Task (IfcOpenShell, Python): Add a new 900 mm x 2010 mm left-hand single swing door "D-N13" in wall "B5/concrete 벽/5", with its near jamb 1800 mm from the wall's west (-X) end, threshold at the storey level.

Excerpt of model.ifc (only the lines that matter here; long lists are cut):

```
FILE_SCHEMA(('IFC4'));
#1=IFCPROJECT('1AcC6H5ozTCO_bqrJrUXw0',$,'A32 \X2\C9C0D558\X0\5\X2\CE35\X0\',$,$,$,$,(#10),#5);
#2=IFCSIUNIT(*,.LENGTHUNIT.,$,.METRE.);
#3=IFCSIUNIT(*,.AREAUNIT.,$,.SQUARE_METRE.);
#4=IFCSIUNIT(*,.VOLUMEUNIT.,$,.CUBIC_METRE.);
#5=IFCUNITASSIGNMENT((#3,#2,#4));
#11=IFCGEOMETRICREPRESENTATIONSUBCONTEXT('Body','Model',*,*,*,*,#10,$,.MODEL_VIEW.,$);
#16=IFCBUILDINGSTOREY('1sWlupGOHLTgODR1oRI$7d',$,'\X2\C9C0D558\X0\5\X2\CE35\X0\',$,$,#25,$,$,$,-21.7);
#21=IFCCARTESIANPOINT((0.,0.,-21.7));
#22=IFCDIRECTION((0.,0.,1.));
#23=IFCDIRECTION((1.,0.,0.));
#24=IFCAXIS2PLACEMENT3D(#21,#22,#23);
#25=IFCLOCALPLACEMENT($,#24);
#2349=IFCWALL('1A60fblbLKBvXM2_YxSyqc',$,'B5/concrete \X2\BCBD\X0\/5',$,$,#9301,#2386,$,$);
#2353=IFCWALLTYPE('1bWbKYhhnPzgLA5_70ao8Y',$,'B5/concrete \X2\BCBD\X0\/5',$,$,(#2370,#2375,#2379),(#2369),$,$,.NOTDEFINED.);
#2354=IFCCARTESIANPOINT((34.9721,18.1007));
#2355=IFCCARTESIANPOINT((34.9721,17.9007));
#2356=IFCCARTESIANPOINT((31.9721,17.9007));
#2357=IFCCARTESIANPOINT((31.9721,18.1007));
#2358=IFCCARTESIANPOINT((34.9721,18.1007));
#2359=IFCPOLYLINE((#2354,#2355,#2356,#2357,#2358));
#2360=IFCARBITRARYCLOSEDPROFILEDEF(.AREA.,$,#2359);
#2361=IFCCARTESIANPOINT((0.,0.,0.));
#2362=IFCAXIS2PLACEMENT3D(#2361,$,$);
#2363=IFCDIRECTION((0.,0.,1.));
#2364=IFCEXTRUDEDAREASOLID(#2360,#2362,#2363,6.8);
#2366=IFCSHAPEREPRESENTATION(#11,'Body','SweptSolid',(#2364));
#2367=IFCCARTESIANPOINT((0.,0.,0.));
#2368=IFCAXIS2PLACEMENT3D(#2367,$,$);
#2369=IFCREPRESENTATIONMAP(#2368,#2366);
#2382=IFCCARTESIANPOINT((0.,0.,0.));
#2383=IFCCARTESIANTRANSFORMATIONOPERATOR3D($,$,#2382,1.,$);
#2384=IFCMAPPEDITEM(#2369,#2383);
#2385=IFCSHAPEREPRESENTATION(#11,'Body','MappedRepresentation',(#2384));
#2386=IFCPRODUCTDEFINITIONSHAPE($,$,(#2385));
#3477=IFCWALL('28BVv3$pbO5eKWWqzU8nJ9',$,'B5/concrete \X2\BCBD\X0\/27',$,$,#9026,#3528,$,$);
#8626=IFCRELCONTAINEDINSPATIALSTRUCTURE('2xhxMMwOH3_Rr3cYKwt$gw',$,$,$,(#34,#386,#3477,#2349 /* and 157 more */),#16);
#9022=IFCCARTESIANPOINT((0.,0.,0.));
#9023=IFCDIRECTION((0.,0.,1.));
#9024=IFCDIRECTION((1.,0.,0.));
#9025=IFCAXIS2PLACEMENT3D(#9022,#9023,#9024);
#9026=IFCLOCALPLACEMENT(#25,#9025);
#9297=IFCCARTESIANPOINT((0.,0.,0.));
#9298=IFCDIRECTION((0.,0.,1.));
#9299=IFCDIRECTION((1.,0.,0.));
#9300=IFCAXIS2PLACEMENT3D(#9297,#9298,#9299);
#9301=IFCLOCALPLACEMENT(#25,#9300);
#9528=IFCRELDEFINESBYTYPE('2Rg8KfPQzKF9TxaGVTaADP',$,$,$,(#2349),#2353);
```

```python
import numpy as np
import ifcopenshell
import ifcopenshell.api.feature
import ifcopenshell.api.geometry
import ifcopenshell.api.root
import ifcopenshell.api.spatial
import ifcopenshell.geom
import ifcopenshell.util.element
import ifcopenshell.util.placement
import ifcopenshell.util.representation
import ifcopenshell.util.shape
import ifcopenshell.util.unit

model = ifcopenshell.open("model.ifc")
unit_scale = ifcopenshell.util.unit.calculate_unit_scale(model)
settings = ifcopenshell.geom.settings()


def volume(element):
    """Net volume in cubic metres, openings subtracted."""
    shape = ifcopenshell.geom.create_shape(settings, element)
    return ifcopenshell.util.shape.get_volume(shape.geometry)


wall = model.by_guid("1A60fblbLKBvXM2_YxSyqc")
storey = ifcopenshell.util.element.get_container(wall, ifc_class="IfcBuildingStorey")
context = ifcopenshell.util.representation.get_context(model, "Model", "Body", "MODEL_VIEW")
before = volume(wall)

width, height, from_end, sill = 0.9, 2.01, 1.8, 0.0  # metres

# The wall runs along its own X axis, and the end named is its -X end.
wall_shape = ifcopenshell.geom.create_shape(settings, wall)
x, y, z = ifcopenshell.util.shape.get_vertices(wall_shape.geometry).T
start = x.min() + from_end
face, thickness = float(y.min()), float(y.max() - y.min())
wall_matrix = ifcopenshell.util.placement.get_local_placement(wall.ObjectPlacement)
level = ifcopenshell.util.placement.get_local_placement(storey.ObjectPlacement)[2, 3]


def in_wall(x, y):
    """Placement at x, y metres in the wall's axes, at sill height."""
    matrix = wall_matrix.copy()
    matrix[:, 3] = wall_matrix @ np.array([x / unit_scale, y / unit_scale, 0.0, 1.0])
    matrix[2, 3] = level + sill / unit_scale
    return matrix


# Opening: a box that overshoots both wall faces by 50 mm.
opening = ifcopenshell.api.root.create_entity(model, ifc_class="IfcOpeningElement", predefined_type="OPENING")
box = ifcopenshell.api.geometry.add_wall_representation(
    model, context=context, length=width, height=height, thickness=thickness + 0.1
)
ifcopenshell.api.geometry.assign_representation(model, product=opening, representation=box)
ifcopenshell.api.geometry.edit_object_placement(model, product=opening, matrix=in_wall(start, face - 0.05), is_si=False)
ifcopenshell.api.feature.add_feature(model, feature=opening, element=wall)

door = ifcopenshell.api.root.create_entity(model, ifc_class="IfcDoor", name="D-N13", predefined_type="DOOR")
door.OverallWidth, door.OverallHeight = width / unit_scale, height / unit_scale
door.OperationType = "SINGLE_SWING_LEFT"
body = ifcopenshell.api.geometry.add_door_representation(
    model,
    context=context,
    overall_width=door.OverallWidth,
    overall_height=door.OverallHeight,
    operation_type="SINGLE_SWING_LEFT",
    lining_properties={"LiningDepth": thickness / unit_scale, "ThresholdDepth": thickness / unit_scale},
)
ifcopenshell.api.geometry.assign_representation(model, product=door, representation=body)
ifcopenshell.api.spatial.assign_container(model, products=[door], relating_structure=storey)
ifcopenshell.api.feature.add_filling(model, opening=opening, element=door)

# The lining spans the wall, so the door starts at the wall face.
ifcopenshell.api.geometry.edit_object_placement(model, product=door, matrix=in_wall(start, face), is_si=False)

after = volume(wall)

print(f"wall volume {before:.3f} -> {after:.3f} m3")

model.write("model_edited.ifc")
```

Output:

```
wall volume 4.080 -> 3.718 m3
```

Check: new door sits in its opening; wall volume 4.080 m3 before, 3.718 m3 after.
